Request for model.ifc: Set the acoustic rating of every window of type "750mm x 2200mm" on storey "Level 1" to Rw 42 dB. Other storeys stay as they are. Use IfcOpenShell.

First a look at what the model holds.

```python
import ifcopenshell
import ifcopenshell.util.element

model = ifcopenshell.open("model.ifc")
print(model.schema)
storey = next(s for s in model.by_type("IfcBuildingStorey") if s.Name == "Level 1")
windows = [e for e in ifcopenshell.util.element.get_decomposition(storey) if e.is_a("IfcWindow")]
seen = {}
for e in windows:
    element_type = ifcopenshell.util.element.get_type(e)
    key = (element_type.Name if element_type != e and element_type else None, ifcopenshell.util.element.get_pset(e, "Pset_WindowCommon", "AcousticRating"))
    seen[key] = seen.get(key, 0) + 1
for (name, value), count in sorted(seen.items(), key=str):
    print(count, "x", name, "|", value)
```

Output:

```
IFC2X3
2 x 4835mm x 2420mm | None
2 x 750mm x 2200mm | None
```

```python
import ifcopenshell
import ifcopenshell.api.pset
import ifcopenshell.util.element

model = ifcopenshell.open("model.ifc")

storey = next(s for s in model.by_type("IfcBuildingStorey") if s.Name == "Level 1")
windows = [e for e in ifcopenshell.util.element.get_decomposition(storey) if e.is_a("IfcWindow")]

count = 0
for e in windows:
    element_type = ifcopenshell.util.element.get_type(e)
    if element_type in (None, e) or element_type.Name != "750mm x 2200mm":
        continue
    # add_pset returns the element's existing set when there is one.
    pset = ifcopenshell.api.pset.add_pset(model, product=e, name="Pset_WindowCommon")
    ifcopenshell.api.pset.edit_pset(model, pset=pset, properties={"AcousticRating": "Rw 42 dB"})
    count += 1

print(count, "windows updated")

model.write("model_rev.ifc")
```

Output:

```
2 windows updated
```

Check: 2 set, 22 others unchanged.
